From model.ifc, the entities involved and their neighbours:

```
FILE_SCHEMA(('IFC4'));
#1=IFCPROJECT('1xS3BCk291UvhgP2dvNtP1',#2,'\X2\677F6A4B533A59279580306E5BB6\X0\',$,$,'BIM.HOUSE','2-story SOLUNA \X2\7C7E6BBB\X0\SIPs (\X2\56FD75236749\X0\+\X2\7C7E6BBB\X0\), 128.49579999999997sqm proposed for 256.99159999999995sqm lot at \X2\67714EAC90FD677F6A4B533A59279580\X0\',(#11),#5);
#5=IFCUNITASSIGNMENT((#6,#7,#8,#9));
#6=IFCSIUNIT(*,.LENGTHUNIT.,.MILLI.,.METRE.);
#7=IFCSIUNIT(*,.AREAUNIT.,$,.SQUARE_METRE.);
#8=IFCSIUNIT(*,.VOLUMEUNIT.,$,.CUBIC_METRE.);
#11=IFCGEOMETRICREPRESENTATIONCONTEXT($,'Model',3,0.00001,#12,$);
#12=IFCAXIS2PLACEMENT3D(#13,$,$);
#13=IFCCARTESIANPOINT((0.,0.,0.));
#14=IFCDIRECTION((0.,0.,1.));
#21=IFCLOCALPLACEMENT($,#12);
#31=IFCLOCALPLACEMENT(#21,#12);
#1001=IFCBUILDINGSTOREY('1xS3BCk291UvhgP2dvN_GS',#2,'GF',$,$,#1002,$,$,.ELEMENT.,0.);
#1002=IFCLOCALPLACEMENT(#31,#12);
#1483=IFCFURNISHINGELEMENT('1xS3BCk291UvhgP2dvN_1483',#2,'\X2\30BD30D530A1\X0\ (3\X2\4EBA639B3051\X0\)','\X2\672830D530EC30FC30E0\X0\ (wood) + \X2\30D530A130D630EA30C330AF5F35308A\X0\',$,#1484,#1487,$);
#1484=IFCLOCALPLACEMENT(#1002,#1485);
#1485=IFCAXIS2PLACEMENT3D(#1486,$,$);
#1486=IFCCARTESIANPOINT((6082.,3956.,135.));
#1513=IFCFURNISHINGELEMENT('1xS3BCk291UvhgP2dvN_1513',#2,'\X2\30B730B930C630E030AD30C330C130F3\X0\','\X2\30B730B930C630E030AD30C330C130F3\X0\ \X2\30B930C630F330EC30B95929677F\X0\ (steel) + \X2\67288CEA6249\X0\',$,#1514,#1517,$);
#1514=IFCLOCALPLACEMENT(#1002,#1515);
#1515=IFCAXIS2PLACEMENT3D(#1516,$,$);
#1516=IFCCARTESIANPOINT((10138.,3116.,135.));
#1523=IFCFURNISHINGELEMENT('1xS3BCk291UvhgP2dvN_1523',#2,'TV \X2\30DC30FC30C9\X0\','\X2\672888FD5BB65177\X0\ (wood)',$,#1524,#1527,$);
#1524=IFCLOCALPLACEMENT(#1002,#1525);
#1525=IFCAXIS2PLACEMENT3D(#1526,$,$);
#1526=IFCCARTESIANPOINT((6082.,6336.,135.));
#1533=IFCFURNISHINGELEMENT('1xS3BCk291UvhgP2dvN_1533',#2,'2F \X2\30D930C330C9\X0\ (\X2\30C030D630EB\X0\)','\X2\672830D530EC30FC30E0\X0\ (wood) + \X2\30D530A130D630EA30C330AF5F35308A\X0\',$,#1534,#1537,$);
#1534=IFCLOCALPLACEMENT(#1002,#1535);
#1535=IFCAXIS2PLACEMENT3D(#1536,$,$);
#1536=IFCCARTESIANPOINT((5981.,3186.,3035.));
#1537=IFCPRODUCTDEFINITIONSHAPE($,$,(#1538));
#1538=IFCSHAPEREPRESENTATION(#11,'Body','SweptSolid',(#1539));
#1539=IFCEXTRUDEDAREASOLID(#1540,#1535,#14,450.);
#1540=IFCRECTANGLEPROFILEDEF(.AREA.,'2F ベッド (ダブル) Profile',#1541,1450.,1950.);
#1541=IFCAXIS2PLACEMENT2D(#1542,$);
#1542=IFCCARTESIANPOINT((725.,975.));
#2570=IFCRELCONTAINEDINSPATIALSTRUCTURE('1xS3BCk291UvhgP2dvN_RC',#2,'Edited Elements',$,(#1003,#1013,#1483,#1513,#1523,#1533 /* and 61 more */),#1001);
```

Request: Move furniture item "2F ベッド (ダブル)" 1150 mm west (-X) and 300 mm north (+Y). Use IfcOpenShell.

```python
import ifcopenshell
import ifcopenshell.api.geometry
import ifcopenshell.util.placement

model = ifcopenshell.open("model.ifc")

item = model.by_guid("1xS3BCk291UvhgP2dvN_1533")
matrix = ifcopenshell.util.placement.get_local_placement(item.ObjectPlacement)
matrix[0, 3] -= 1150.0
matrix[1, 3] += 300.0
ifcopenshell.api.geometry.edit_object_placement(model, product=item, matrix=matrix, is_si=False)

print(ifcopenshell.util.placement.get_local_placement(item.ObjectPlacement).round(3) + 0.0)

model.write("model_updated.ifc")
```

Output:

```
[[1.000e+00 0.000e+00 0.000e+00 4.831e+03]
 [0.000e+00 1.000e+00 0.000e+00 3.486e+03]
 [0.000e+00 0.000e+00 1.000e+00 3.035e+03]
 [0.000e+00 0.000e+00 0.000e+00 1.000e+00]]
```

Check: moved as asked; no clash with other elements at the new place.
